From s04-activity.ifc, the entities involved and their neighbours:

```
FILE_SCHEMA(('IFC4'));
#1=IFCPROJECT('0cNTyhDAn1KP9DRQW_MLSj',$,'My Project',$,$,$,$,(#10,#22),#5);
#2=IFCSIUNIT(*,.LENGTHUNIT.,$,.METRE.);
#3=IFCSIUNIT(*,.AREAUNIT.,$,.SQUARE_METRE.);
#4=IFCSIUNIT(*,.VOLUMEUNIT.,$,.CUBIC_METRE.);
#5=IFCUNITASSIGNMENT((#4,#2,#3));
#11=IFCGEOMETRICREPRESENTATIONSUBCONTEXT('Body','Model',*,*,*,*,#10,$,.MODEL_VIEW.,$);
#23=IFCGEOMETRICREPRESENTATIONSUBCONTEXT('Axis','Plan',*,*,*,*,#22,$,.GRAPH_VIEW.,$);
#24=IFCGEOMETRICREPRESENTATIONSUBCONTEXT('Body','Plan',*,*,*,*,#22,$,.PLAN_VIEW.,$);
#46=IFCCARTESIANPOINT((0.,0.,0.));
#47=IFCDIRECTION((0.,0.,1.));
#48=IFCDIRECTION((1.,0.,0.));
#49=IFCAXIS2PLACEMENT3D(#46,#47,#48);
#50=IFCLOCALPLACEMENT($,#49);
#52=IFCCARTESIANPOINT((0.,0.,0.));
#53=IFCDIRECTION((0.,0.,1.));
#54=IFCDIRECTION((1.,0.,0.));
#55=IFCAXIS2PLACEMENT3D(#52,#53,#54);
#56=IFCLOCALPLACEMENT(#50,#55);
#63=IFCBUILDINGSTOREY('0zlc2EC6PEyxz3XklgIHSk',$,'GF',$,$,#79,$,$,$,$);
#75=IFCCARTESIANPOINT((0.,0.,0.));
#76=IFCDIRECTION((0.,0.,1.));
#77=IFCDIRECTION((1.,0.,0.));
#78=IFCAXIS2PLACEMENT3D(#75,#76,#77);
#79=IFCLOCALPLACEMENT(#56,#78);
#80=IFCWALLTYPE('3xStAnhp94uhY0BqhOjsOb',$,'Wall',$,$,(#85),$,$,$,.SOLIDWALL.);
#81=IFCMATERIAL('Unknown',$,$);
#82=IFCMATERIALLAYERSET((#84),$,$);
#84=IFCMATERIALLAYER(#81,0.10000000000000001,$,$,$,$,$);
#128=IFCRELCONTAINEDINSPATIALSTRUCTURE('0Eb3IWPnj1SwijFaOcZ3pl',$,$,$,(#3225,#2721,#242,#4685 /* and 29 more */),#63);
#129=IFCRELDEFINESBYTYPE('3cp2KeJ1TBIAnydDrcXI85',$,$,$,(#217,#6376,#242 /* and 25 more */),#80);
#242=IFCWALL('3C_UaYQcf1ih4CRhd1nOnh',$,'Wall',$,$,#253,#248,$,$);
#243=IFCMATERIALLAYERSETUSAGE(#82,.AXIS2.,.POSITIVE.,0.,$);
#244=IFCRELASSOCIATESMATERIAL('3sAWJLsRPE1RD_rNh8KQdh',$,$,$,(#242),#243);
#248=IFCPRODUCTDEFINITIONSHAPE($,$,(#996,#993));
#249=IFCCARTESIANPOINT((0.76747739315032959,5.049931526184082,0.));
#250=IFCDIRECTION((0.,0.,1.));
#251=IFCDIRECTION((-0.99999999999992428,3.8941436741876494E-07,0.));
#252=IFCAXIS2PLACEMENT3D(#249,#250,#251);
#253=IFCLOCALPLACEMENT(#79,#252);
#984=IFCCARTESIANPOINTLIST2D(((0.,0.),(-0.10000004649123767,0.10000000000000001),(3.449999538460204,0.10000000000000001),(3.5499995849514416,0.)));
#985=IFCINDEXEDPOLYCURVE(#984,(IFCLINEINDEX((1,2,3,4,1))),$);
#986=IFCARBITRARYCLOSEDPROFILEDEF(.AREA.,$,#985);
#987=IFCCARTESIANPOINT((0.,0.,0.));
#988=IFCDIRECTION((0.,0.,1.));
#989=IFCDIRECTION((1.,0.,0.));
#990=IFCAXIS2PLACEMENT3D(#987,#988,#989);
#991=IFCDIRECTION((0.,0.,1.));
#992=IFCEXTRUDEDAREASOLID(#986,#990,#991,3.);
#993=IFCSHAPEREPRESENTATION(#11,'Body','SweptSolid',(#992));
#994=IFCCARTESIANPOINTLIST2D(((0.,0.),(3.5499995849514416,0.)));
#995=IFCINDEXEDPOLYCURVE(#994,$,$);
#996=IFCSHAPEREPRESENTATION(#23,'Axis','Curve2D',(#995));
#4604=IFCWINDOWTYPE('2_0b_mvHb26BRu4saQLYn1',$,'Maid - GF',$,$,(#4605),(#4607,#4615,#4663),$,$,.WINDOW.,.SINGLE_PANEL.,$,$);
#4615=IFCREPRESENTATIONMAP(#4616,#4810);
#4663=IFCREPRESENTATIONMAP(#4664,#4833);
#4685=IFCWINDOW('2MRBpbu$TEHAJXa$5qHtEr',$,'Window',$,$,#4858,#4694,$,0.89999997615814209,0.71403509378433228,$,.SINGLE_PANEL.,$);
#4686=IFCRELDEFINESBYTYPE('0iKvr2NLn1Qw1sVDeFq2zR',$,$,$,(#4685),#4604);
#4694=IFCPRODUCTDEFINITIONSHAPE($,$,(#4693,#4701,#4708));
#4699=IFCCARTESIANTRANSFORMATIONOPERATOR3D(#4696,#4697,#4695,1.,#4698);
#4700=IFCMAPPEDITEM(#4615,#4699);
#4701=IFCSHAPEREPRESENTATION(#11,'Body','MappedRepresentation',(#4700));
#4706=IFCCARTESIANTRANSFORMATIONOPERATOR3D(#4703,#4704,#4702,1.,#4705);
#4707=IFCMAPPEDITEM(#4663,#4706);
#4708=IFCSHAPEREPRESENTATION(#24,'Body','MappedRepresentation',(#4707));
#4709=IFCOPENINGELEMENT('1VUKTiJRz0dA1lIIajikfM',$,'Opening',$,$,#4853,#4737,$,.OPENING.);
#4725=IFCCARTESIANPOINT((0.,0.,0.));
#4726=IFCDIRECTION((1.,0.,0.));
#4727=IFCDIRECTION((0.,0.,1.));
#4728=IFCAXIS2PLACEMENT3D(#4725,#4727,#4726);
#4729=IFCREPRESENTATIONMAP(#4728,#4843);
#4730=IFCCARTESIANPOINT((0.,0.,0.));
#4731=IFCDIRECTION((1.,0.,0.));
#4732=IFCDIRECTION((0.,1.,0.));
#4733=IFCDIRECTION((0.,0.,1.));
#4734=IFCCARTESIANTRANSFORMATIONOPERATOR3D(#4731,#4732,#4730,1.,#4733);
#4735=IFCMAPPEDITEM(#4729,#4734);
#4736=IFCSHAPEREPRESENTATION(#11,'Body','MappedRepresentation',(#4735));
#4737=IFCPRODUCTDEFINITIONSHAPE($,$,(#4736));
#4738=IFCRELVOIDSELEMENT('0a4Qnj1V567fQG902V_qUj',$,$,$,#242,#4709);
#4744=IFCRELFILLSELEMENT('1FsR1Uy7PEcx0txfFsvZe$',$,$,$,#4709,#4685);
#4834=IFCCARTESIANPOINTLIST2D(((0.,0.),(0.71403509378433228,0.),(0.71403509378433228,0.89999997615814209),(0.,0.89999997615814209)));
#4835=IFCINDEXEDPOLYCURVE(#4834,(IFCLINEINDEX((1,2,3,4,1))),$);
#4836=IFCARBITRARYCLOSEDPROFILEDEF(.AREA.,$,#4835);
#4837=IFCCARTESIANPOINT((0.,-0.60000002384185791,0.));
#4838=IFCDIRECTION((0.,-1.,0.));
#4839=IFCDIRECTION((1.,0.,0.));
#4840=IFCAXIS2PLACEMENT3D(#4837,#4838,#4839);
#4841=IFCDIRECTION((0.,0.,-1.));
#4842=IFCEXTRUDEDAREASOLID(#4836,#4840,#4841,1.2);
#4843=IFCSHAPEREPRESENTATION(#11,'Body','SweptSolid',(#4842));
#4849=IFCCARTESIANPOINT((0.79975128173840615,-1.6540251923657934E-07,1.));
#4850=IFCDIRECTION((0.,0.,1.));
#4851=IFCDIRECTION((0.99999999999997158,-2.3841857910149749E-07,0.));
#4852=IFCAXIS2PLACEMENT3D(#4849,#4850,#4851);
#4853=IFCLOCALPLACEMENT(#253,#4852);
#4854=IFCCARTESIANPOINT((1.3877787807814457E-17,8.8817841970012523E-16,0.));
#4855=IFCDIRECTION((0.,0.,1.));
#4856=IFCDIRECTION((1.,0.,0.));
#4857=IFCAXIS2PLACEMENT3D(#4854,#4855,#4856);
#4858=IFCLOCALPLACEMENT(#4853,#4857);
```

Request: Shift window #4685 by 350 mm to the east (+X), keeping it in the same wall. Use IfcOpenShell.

```python
import ifcopenshell
import ifcopenshell.api.geometry
import ifcopenshell.util.placement
import ifcopenshell.util.unit

model = ifcopenshell.open("s04-activity.ifc")
unit_scale = ifcopenshell.util.unit.calculate_unit_scale(model)

window = model.by_guid("2MRBpbu$TEHAJXa$5qHtEr")
opening = window.FillsVoids[0].RelatingOpeningElement
wall = opening.VoidsElements[0].RelatingBuildingElement

wall_matrix = ifcopenshell.util.placement.get_local_placement(wall.ObjectPlacement)
shift = wall_matrix[:3, 0] * -0.35 / unit_scale
before = ifcopenshell.util.placement.get_local_placement(window.ObjectPlacement)[:3, 3].copy()

# The window is placed relative to its opening, so it follows when the opening moves.
matrix = ifcopenshell.util.placement.get_local_placement(opening.ObjectPlacement)
matrix[:3, 3] += shift
ifcopenshell.api.geometry.edit_object_placement(
    model, product=opening, matrix=matrix, is_si=False, should_transform_children=True
)

after = ifcopenshell.util.placement.get_local_placement(window.ObjectPlacement)[:3, 3]
print("window moved by", (after - before).round(3) + 0.0)

model.write("s04-activity_v2.ifc")
```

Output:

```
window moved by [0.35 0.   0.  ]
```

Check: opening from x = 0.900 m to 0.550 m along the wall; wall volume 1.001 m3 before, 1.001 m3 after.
